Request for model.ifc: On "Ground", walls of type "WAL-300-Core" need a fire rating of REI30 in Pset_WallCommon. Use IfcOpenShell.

First a look at what the model holds.

```python
import ifcopenshell
import ifcopenshell.util.element

model = ifcopenshell.open("model.ifc")
print(model.schema)
storey = next(s for s in model.by_type("IfcBuildingStorey") if s.Name == "Ground")
walls = [e for e in ifcopenshell.util.element.get_decomposition(storey) if e.is_a("IfcWall")]
seen = {}
for e in walls:
    element_type = ifcopenshell.util.element.get_type(e)
    key = (element_type.Name if element_type != e and element_type else None, ifcopenshell.util.element.get_pset(e, "Pset_WallCommon", "FireRating"))
    seen[key] = seen.get(key, 0) + 1
for (name, value), count in sorted(seen.items(), key=str):
    print(count, "x", name, "|", value)
```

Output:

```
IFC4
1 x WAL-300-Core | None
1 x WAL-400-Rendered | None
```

```python
import ifcopenshell
import ifcopenshell.api.pset
import ifcopenshell.util.element

model = ifcopenshell.open("model.ifc")

storey = next(s for s in model.by_type("IfcBuildingStorey") if s.Name == "Ground")
walls = [e for e in ifcopenshell.util.element.get_decomposition(storey) if e.is_a("IfcWall")]

count = 0
for e in walls:
    element_type = ifcopenshell.util.element.get_type(e)
    if element_type in (None, e) or element_type.Name != "WAL-300-Core":
        continue
    # add_pset returns the element's existing set when there is one.
    pset = ifcopenshell.api.pset.add_pset(model, product=e, name="Pset_WallCommon")
    ifcopenshell.api.pset.edit_pset(model, pset=pset, properties={"FireRating": "REI30"})
    count += 1

print(count, "walls updated")

model.write("model_v2.ifc")
```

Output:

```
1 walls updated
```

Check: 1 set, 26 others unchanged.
